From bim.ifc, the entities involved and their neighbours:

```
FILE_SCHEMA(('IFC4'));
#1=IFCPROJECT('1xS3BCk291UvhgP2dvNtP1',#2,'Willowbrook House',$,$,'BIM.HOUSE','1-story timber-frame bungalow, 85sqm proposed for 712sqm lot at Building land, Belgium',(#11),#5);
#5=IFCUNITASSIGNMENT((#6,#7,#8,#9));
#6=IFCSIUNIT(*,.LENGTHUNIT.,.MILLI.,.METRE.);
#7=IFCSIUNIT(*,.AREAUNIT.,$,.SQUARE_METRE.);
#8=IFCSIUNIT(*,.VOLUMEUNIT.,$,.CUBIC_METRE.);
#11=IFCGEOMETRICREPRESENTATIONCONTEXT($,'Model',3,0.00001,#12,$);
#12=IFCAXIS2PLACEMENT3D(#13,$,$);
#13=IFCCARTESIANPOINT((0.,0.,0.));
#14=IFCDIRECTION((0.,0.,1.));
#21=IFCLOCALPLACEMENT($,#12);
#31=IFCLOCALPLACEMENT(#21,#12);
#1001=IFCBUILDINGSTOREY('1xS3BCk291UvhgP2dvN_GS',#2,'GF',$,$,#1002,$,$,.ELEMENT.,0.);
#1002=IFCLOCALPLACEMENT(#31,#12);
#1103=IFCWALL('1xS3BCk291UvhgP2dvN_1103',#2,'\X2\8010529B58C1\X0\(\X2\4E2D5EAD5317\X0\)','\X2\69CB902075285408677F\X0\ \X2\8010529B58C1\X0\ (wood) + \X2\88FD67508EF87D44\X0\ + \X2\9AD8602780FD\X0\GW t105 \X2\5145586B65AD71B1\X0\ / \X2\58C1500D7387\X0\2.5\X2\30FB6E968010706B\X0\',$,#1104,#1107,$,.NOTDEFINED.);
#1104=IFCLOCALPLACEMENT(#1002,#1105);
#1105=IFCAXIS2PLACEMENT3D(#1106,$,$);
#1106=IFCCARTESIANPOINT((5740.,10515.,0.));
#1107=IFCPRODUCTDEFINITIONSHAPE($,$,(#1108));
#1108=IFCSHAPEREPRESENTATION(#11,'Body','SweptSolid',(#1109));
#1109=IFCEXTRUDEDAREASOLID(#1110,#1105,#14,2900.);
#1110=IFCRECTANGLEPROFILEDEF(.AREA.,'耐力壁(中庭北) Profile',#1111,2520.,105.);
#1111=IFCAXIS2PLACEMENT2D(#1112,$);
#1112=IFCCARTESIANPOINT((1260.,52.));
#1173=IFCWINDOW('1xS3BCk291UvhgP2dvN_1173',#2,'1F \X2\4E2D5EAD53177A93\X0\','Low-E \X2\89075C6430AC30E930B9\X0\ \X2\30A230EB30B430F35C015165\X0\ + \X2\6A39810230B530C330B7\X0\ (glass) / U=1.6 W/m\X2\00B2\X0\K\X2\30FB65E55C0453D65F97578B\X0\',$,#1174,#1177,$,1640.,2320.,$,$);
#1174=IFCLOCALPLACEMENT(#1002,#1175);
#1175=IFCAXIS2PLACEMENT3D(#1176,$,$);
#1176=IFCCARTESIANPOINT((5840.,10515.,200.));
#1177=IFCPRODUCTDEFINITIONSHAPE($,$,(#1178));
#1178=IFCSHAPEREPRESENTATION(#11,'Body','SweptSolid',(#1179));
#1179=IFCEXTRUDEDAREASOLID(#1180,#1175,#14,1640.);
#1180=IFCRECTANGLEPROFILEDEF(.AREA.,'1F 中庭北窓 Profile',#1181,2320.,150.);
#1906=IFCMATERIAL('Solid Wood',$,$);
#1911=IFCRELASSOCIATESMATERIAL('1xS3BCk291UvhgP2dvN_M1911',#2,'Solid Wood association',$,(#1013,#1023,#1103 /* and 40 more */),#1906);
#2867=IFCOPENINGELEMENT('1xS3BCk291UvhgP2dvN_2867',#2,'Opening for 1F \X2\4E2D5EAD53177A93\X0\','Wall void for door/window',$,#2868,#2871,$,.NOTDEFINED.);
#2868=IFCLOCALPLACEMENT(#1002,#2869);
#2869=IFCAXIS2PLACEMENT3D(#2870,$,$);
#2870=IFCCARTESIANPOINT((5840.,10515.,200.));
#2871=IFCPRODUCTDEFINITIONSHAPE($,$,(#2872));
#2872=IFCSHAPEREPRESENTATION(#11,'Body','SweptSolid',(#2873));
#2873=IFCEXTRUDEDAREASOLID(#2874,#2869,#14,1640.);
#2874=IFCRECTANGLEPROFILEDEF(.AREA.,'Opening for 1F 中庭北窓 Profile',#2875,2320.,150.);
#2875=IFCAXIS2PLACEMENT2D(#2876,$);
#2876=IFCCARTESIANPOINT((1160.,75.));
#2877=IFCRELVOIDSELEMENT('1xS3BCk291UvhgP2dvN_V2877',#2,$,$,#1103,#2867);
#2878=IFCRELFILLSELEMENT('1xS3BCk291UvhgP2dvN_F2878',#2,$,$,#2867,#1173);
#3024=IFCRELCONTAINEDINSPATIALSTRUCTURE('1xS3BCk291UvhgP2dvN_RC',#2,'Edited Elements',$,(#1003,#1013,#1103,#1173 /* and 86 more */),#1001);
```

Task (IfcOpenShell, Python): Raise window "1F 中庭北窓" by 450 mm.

```python
import numpy as np
import ifcopenshell
import ifcopenshell.api.geometry
import ifcopenshell.util.placement
import ifcopenshell.util.unit

model = ifcopenshell.open("bim.ifc")
unit_scale = ifcopenshell.util.unit.calculate_unit_scale(model)

window = model.by_id(1173)
opening = window.FillsVoids[0].RelatingOpeningElement
dz = 450.0

shift = np.array([0.0, 0.0, dz])
# The window is not placed relative to its opening, so move both.
for product in (opening, window):
    matrix = ifcopenshell.util.placement.get_local_placement(product.ObjectPlacement)
    matrix[:3, 3] += shift
    ifcopenshell.api.geometry.edit_object_placement(model, product=product, matrix=matrix, is_si=False)

print(f"moved by {dz * unit_scale:+.3f} m")

model.write("bim-out.ifc")
```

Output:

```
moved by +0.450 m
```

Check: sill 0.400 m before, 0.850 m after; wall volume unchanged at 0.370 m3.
